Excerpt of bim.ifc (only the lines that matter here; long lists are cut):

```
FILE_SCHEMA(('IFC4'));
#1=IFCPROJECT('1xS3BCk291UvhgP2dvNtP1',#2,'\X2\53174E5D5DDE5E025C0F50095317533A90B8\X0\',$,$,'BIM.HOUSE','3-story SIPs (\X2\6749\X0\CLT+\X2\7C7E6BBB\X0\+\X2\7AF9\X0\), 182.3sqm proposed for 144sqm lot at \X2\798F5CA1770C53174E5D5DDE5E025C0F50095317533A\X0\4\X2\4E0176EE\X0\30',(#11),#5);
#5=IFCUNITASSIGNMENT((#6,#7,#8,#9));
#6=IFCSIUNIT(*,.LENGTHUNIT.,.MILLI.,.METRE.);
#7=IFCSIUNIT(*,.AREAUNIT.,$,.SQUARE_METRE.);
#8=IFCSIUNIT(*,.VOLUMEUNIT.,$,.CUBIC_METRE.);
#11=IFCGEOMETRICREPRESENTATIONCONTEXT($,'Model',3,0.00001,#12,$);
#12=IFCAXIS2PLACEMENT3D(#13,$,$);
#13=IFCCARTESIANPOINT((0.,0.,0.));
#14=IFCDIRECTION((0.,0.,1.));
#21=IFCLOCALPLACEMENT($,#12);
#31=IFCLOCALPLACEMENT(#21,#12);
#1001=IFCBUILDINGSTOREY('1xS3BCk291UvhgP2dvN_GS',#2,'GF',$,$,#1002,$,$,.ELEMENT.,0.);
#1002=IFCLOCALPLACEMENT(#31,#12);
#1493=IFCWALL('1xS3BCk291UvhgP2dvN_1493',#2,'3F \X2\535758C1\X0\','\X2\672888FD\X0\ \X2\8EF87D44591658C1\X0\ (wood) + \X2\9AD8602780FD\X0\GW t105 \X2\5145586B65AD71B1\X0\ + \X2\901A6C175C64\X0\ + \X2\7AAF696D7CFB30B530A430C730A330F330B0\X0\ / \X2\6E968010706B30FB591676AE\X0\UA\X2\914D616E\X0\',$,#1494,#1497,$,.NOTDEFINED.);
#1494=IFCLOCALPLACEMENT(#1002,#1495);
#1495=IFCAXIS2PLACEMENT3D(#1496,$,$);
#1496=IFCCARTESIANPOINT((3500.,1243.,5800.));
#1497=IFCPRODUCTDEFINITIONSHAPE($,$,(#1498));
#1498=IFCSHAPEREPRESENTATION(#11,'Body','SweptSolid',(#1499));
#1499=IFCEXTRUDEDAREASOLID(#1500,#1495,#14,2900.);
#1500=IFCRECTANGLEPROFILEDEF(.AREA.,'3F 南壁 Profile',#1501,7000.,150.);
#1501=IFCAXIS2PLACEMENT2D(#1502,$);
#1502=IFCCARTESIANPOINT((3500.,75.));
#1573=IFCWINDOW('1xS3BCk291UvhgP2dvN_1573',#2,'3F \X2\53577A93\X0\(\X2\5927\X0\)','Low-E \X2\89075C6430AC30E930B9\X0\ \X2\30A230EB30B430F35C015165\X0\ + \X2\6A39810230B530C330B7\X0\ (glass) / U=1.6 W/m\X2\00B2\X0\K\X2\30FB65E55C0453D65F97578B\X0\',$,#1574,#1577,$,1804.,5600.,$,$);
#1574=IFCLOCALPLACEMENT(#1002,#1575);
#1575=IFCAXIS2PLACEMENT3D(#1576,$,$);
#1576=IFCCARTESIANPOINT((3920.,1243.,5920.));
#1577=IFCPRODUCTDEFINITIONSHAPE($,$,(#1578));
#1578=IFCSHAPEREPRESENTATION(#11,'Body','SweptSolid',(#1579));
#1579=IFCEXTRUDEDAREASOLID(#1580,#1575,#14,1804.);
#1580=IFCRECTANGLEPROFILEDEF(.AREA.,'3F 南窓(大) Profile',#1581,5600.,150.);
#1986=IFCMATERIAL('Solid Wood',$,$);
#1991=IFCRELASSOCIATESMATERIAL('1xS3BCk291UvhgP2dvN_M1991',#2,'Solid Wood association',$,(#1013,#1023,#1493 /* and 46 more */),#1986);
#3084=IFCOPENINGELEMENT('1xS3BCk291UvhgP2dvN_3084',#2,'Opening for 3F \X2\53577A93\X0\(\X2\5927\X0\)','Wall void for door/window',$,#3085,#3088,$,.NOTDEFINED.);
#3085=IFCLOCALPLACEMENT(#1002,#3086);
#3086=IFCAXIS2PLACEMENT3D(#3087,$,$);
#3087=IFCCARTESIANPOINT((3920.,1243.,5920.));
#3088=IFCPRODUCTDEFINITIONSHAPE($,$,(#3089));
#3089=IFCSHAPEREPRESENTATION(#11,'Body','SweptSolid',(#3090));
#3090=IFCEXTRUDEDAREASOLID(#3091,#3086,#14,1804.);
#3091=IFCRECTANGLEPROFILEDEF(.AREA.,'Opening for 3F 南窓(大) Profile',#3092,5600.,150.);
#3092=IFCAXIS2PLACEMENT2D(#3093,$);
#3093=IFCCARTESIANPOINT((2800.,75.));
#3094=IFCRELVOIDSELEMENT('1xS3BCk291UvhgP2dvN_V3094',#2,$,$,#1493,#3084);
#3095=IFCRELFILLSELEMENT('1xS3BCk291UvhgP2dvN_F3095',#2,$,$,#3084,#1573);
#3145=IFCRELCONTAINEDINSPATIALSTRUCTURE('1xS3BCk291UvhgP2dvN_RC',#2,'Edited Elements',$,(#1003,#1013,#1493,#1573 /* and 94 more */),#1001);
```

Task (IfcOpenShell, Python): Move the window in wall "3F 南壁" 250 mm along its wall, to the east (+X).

```python
import ifcopenshell
import ifcopenshell.api.geometry
import ifcopenshell.util.placement

model = ifcopenshell.open("bim.ifc")

window = model.by_guid("1xS3BCk291UvhgP2dvN_1573")
opening = window.FillsVoids[0].RelatingOpeningElement
wall = opening.VoidsElements[0].RelatingBuildingElement

wall_matrix = ifcopenshell.util.placement.get_local_placement(wall.ObjectPlacement)
shift = wall_matrix[:3, 0] * 250.0
before = ifcopenshell.util.placement.get_local_placement(window.ObjectPlacement)[:3, 3].copy()

# The window is not placed relative to its opening, so move both.
for product in (opening, window):
    matrix = ifcopenshell.util.placement.get_local_placement(product.ObjectPlacement)
    matrix[:3, 3] += shift
    ifcopenshell.api.geometry.edit_object_placement(model, product=product, matrix=matrix, is_si=False)

after = ifcopenshell.util.placement.get_local_placement(window.ObjectPlacement)[:3, 3]
print("window moved by", (after - before).round(3) + 0.0)

model.write("bim-out.ifc")
```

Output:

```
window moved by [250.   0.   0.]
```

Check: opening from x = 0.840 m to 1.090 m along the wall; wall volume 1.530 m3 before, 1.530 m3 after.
